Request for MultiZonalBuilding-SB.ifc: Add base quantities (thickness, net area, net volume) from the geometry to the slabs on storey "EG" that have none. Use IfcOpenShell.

First a look at what the model holds.

```python
import ifcopenshell
import ifcopenshell.util.element
import ifcopenshell.util.unit

model = ifcopenshell.open("MultiZonalBuilding-SB.ifc")
print(model.schema)
for unit_type in ("LENGTHUNIT", "AREAUNIT", "VOLUMEUNIT"):
    print(unit_type, ifcopenshell.util.unit.calculate_unit_scale(model, unit_type))
storey = next(s for s in model.by_type("IfcBuildingStorey") if s.Name == "EG")
slabs = [e for e in ifcopenshell.util.element.get_decomposition(storey) if e.is_a("IfcSlab")]
for e in sorted(slabs, key=lambda e: e.id()):
    print(e.id(), e.is_a(), e.Name, list(ifcopenshell.util.element.get_psets(e, qtos_only=True)), sep=" | ")
```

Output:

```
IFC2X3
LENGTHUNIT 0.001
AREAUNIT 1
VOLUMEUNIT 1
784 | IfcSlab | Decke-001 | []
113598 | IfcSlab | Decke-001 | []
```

```python
import ifcopenshell
import ifcopenshell.api.pset
import ifcopenshell.geom
import ifcopenshell.util.element
import ifcopenshell.util.shape
import ifcopenshell.util.unit

model = ifcopenshell.open("MultiZonalBuilding-SB.ifc")
unit_scale = ifcopenshell.util.unit.calculate_unit_scale(model)
area_scale = ifcopenshell.util.unit.calculate_unit_scale(model, "AREAUNIT")
volume_scale = ifcopenshell.util.unit.calculate_unit_scale(model, "VOLUMEUNIT")
settings = ifcopenshell.geom.settings()

storey = next(s for s in model.by_type("IfcBuildingStorey") if s.Name == "EG")
slabs = [e for e in ifcopenshell.util.element.get_decomposition(storey) if e.is_a("IfcSlab")]

for e in sorted(slabs, key=lambda e: e.id()):
    if ifcopenshell.util.element.get_psets(e, qtos_only=True, should_inherit=False):
        continue
    # Geometry comes back in metres, in the element's own axes.
    shape = ifcopenshell.geom.create_shape(settings, e)
    values = {
        "Width": ifcopenshell.util.shape.get_z(shape.geometry) / unit_scale,
        "NetArea": ifcopenshell.util.shape.get_footprint_area(shape.geometry) / area_scale,
        "NetVolume": ifcopenshell.util.shape.get_volume(shape.geometry) / volume_scale,
    }
    qto = ifcopenshell.api.pset.add_qto(model, product=e, name="BaseQuantities")
    ifcopenshell.api.pset.edit_qto(model, qto=qto, properties=values)
    print(e.id(), {k: round(v, 3) for k, v in values.items()})

model.write("MultiZonalBuilding-SB_v2.ifc")
```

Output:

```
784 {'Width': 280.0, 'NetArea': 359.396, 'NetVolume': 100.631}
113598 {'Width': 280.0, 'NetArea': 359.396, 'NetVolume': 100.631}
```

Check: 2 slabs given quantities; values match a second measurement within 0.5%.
